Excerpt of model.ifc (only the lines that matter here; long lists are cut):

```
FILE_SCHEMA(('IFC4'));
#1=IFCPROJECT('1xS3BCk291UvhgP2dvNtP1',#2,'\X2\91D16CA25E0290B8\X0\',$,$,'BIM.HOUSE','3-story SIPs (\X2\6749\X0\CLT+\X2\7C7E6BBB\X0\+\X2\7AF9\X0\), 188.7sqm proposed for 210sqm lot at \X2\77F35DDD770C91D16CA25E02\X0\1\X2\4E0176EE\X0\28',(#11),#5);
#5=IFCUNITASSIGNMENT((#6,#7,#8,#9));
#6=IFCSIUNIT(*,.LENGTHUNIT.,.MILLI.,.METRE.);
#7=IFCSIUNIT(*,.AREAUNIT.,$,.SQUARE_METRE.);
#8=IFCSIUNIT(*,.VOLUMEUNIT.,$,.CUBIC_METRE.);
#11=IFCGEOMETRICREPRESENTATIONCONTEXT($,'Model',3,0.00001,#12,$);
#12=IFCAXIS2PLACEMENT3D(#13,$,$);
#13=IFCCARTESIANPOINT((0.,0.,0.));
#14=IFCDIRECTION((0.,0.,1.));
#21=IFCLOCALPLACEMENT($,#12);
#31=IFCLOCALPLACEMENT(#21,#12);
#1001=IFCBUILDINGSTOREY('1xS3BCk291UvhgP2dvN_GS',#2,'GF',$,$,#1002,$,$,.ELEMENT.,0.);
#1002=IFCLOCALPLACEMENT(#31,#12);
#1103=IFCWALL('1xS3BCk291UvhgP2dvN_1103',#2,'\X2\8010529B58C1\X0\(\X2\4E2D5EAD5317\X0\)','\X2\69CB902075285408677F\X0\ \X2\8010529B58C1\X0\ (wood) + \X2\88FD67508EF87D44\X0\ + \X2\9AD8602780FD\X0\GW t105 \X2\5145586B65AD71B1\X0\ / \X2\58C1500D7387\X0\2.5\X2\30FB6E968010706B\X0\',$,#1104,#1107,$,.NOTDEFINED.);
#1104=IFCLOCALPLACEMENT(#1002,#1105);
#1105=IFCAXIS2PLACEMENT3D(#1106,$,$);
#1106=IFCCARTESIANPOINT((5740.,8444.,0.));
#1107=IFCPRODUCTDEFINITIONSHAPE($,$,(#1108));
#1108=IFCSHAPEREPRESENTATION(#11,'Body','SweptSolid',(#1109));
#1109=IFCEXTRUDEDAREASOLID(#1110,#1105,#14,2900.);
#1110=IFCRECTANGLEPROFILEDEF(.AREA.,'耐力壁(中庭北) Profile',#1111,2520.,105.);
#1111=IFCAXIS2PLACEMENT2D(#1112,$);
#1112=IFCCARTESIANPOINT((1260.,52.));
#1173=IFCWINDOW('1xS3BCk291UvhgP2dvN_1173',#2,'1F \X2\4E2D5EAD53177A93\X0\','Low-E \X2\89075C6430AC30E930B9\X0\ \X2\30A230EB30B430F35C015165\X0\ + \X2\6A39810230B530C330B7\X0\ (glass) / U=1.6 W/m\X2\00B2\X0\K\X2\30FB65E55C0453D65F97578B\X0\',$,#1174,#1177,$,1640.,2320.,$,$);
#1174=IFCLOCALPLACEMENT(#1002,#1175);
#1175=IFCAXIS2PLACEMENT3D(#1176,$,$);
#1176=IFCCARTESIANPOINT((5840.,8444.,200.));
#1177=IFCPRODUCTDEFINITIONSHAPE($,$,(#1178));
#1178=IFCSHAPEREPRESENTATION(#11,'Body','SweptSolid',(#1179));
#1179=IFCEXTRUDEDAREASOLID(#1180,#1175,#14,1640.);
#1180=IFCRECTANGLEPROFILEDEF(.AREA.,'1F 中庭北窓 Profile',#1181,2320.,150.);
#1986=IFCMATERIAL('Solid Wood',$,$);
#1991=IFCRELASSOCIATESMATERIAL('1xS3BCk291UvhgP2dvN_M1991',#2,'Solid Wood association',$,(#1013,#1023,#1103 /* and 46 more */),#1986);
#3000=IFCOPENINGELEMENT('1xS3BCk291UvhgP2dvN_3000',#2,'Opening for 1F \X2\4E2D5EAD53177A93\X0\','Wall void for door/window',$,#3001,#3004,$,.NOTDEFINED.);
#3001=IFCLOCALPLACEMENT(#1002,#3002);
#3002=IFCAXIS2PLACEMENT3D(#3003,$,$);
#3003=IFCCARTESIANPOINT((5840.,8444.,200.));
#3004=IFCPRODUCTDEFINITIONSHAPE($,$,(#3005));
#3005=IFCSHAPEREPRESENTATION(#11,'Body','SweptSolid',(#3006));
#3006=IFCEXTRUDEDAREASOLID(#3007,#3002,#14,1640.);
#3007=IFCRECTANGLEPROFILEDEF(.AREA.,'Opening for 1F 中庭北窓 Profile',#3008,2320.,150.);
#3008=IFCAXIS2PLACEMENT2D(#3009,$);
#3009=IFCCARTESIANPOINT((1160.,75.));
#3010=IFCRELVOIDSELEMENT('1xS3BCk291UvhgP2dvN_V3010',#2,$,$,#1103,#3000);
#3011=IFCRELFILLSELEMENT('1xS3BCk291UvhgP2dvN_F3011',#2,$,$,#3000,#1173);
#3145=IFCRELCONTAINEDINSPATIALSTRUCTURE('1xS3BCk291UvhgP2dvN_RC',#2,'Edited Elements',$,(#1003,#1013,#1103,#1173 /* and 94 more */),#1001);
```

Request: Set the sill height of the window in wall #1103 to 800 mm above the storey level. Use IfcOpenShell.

```python
import numpy as np
import ifcopenshell
import ifcopenshell.api.geometry
import ifcopenshell.geom
import ifcopenshell.util.element
import ifcopenshell.util.placement
import ifcopenshell.util.shape
import ifcopenshell.util.unit

model = ifcopenshell.open("model.ifc")
unit_scale = ifcopenshell.util.unit.calculate_unit_scale(model)

window = model.by_guid("1xS3BCk291UvhgP2dvN_1173")
opening = window.FillsVoids[0].RelatingOpeningElement
storey = ifcopenshell.util.element.get_container(window, ifc_class="IfcBuildingStorey")
level = ifcopenshell.util.placement.get_local_placement(storey.ObjectPlacement)[2, 3]

# The opening's origin need not be at the sill, so measure its lowest point.
shape = ifcopenshell.geom.create_shape(ifcopenshell.geom.settings(), opening)
bottom = ifcopenshell.util.shape.get_shape_bottom_elevation(shape, shape.geometry) / unit_scale
dz = level + 0.8 / unit_scale - bottom

shift = np.array([0.0, 0.0, dz])
# The window is not placed relative to its opening, so move both.
for product in (opening, window):
    matrix = ifcopenshell.util.placement.get_local_placement(product.ObjectPlacement)
    matrix[:3, 3] += shift
    ifcopenshell.api.geometry.edit_object_placement(model, product=product, matrix=matrix, is_si=False)

print(f"moved by {dz * unit_scale:+.3f} m")

model.write("model_v2.ifc")
```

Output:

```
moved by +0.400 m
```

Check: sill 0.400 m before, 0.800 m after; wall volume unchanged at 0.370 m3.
